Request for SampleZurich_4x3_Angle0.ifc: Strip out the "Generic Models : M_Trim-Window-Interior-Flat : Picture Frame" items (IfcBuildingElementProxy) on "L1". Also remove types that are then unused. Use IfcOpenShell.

First a look at what the model holds.

```python
import ifcopenshell
import ifcopenshell.util.element

model = ifcopenshell.open("SampleZurich_4x3_Angle0.ifc")
print(model.schema)
storey = next(s for s in model.by_type("IfcBuildingStorey") if s.Name == "L1")
proxies = [e for e in ifcopenshell.util.element.get_decomposition(storey) if e.is_a("IfcBuildingElementProxy")]
seen = {}
for e in proxies:
    element_type = ifcopenshell.util.element.get_type(e)
    name = element_type.Name if element_type not in (None, e) else None
    seen[name] = seen.get(name, 0) + 1
for name, count in sorted(seen.items(), key=str):
    print(count, "x", name)
```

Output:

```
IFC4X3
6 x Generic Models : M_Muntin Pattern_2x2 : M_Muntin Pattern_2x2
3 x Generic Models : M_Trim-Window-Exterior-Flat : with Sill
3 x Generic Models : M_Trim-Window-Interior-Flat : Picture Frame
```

```python
import ifcopenshell
import ifcopenshell.api.root
import ifcopenshell.util.element

model = ifcopenshell.open("SampleZurich_4x3_Angle0.ifc")

storey = next(s for s in model.by_type("IfcBuildingStorey") if s.Name == "L1")
proxies = [e for e in ifcopenshell.util.element.get_decomposition(storey) if e.is_a("IfcBuildingElementProxy")]
targets = [e for e in proxies if (t := ifcopenshell.util.element.get_type(e)) not in (None, e) and t.Name == "Generic Models : M_Trim-Window-Interior-Flat : Picture Frame"]
types = {ifcopenshell.util.element.get_type(e) for e in targets} - {None, *targets}

for e in targets:
    ifcopenshell.api.root.remove_product(model, product=e)
print(len(targets), "removed")

unused = [t for t in types if not ifcopenshell.util.element.get_types(t)]
for t in unused:
    ifcopenshell.api.root.remove_product(model, product=t)
print(len(unused), "unused types removed")

model.write("SampleZurich_4x3_Angle0_edited.ifc")
```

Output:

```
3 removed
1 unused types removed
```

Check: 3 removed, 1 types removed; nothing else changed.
